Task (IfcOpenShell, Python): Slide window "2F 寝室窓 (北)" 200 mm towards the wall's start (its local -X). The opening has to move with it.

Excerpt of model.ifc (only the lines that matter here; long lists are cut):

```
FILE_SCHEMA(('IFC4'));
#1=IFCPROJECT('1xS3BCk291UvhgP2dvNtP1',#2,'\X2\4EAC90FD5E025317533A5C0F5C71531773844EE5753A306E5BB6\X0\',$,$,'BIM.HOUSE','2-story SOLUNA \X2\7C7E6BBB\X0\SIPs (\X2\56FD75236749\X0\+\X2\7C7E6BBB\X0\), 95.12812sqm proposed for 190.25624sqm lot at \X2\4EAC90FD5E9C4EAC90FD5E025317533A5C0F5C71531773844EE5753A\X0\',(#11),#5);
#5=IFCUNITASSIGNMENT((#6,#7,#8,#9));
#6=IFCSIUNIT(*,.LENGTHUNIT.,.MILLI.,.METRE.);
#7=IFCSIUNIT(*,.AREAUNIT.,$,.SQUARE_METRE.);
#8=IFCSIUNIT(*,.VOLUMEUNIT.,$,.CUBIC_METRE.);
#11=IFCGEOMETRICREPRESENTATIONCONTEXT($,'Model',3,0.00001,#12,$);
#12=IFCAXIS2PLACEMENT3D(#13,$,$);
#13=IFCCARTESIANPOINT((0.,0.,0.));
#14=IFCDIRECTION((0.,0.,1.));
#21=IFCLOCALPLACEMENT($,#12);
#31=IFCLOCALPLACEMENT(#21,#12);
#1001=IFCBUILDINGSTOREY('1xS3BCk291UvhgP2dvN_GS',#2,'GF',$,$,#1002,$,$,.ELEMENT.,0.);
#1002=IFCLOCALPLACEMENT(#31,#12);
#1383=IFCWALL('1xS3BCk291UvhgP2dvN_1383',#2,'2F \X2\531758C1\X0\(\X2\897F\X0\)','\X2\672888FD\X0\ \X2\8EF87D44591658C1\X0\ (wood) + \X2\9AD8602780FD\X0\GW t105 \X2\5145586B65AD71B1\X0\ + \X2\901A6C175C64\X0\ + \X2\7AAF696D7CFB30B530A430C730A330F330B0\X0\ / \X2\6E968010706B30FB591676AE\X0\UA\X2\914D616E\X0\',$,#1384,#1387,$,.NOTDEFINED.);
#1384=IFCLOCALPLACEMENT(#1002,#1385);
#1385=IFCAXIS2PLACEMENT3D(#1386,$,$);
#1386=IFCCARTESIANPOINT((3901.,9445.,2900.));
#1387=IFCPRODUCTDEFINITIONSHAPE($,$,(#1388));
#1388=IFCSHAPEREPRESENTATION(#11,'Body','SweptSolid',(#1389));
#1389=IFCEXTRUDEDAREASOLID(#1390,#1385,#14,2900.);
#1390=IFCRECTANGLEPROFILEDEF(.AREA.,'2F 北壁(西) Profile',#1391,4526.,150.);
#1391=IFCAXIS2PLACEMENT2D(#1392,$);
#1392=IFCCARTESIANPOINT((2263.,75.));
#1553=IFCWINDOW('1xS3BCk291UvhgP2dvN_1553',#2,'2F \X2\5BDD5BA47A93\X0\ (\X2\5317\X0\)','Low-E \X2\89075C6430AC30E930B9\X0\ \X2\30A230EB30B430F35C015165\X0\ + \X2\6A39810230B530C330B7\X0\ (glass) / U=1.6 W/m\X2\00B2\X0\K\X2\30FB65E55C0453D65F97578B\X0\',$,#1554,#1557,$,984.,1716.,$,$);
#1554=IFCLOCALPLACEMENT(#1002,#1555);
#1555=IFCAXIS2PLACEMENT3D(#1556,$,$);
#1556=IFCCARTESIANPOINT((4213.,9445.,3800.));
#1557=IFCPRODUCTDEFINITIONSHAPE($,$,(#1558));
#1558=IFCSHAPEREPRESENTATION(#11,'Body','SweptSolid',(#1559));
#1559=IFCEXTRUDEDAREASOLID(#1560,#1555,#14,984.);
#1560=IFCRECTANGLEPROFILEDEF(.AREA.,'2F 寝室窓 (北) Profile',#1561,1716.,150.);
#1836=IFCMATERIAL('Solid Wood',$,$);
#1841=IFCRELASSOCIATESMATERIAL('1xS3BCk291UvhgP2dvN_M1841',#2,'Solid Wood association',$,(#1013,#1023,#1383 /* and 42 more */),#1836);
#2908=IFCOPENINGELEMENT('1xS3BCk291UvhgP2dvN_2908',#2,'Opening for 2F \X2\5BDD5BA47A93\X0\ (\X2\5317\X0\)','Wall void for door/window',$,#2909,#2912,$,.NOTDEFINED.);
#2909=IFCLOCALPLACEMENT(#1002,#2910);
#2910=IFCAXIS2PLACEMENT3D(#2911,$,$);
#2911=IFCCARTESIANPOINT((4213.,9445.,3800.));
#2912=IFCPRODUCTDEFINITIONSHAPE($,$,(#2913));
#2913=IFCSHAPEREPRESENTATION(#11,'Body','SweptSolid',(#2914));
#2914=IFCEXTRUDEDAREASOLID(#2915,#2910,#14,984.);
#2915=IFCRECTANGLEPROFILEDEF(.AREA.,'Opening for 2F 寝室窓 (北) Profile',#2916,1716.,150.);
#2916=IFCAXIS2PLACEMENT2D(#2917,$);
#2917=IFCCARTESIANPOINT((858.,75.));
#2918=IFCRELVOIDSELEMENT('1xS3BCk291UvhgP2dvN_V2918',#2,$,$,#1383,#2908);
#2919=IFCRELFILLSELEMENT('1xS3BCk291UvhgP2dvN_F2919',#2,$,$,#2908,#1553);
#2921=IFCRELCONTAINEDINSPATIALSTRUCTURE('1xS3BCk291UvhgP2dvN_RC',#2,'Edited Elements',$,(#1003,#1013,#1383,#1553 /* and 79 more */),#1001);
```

```python
import ifcopenshell
import ifcopenshell.api.geometry
import ifcopenshell.util.placement
import ifcopenshell.util.unit

model = ifcopenshell.open("model.ifc")
unit_scale = ifcopenshell.util.unit.calculate_unit_scale(model)

window = model.by_guid("1xS3BCk291UvhgP2dvN_1553")
opening = window.FillsVoids[0].RelatingOpeningElement
wall = opening.VoidsElements[0].RelatingBuildingElement

wall_matrix = ifcopenshell.util.placement.get_local_placement(wall.ObjectPlacement)
shift = wall_matrix[:3, 0] * -0.2 / unit_scale
before = ifcopenshell.util.placement.get_local_placement(window.ObjectPlacement)[:3, 3].copy()

# The window is not placed relative to its opening, so move both.
for product in (opening, window):
    matrix = ifcopenshell.util.placement.get_local_placement(product.ObjectPlacement)
    matrix[:3, 3] += shift
    ifcopenshell.api.geometry.edit_object_placement(model, product=product, matrix=matrix, is_si=False)

after = ifcopenshell.util.placement.get_local_placement(window.ObjectPlacement)[:3, 3]
print("window moved by", (after - before).round(3) + 0.0)

model.write("model_rev.ifc")
```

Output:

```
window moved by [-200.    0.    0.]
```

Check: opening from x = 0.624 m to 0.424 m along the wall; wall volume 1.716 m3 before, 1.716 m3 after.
